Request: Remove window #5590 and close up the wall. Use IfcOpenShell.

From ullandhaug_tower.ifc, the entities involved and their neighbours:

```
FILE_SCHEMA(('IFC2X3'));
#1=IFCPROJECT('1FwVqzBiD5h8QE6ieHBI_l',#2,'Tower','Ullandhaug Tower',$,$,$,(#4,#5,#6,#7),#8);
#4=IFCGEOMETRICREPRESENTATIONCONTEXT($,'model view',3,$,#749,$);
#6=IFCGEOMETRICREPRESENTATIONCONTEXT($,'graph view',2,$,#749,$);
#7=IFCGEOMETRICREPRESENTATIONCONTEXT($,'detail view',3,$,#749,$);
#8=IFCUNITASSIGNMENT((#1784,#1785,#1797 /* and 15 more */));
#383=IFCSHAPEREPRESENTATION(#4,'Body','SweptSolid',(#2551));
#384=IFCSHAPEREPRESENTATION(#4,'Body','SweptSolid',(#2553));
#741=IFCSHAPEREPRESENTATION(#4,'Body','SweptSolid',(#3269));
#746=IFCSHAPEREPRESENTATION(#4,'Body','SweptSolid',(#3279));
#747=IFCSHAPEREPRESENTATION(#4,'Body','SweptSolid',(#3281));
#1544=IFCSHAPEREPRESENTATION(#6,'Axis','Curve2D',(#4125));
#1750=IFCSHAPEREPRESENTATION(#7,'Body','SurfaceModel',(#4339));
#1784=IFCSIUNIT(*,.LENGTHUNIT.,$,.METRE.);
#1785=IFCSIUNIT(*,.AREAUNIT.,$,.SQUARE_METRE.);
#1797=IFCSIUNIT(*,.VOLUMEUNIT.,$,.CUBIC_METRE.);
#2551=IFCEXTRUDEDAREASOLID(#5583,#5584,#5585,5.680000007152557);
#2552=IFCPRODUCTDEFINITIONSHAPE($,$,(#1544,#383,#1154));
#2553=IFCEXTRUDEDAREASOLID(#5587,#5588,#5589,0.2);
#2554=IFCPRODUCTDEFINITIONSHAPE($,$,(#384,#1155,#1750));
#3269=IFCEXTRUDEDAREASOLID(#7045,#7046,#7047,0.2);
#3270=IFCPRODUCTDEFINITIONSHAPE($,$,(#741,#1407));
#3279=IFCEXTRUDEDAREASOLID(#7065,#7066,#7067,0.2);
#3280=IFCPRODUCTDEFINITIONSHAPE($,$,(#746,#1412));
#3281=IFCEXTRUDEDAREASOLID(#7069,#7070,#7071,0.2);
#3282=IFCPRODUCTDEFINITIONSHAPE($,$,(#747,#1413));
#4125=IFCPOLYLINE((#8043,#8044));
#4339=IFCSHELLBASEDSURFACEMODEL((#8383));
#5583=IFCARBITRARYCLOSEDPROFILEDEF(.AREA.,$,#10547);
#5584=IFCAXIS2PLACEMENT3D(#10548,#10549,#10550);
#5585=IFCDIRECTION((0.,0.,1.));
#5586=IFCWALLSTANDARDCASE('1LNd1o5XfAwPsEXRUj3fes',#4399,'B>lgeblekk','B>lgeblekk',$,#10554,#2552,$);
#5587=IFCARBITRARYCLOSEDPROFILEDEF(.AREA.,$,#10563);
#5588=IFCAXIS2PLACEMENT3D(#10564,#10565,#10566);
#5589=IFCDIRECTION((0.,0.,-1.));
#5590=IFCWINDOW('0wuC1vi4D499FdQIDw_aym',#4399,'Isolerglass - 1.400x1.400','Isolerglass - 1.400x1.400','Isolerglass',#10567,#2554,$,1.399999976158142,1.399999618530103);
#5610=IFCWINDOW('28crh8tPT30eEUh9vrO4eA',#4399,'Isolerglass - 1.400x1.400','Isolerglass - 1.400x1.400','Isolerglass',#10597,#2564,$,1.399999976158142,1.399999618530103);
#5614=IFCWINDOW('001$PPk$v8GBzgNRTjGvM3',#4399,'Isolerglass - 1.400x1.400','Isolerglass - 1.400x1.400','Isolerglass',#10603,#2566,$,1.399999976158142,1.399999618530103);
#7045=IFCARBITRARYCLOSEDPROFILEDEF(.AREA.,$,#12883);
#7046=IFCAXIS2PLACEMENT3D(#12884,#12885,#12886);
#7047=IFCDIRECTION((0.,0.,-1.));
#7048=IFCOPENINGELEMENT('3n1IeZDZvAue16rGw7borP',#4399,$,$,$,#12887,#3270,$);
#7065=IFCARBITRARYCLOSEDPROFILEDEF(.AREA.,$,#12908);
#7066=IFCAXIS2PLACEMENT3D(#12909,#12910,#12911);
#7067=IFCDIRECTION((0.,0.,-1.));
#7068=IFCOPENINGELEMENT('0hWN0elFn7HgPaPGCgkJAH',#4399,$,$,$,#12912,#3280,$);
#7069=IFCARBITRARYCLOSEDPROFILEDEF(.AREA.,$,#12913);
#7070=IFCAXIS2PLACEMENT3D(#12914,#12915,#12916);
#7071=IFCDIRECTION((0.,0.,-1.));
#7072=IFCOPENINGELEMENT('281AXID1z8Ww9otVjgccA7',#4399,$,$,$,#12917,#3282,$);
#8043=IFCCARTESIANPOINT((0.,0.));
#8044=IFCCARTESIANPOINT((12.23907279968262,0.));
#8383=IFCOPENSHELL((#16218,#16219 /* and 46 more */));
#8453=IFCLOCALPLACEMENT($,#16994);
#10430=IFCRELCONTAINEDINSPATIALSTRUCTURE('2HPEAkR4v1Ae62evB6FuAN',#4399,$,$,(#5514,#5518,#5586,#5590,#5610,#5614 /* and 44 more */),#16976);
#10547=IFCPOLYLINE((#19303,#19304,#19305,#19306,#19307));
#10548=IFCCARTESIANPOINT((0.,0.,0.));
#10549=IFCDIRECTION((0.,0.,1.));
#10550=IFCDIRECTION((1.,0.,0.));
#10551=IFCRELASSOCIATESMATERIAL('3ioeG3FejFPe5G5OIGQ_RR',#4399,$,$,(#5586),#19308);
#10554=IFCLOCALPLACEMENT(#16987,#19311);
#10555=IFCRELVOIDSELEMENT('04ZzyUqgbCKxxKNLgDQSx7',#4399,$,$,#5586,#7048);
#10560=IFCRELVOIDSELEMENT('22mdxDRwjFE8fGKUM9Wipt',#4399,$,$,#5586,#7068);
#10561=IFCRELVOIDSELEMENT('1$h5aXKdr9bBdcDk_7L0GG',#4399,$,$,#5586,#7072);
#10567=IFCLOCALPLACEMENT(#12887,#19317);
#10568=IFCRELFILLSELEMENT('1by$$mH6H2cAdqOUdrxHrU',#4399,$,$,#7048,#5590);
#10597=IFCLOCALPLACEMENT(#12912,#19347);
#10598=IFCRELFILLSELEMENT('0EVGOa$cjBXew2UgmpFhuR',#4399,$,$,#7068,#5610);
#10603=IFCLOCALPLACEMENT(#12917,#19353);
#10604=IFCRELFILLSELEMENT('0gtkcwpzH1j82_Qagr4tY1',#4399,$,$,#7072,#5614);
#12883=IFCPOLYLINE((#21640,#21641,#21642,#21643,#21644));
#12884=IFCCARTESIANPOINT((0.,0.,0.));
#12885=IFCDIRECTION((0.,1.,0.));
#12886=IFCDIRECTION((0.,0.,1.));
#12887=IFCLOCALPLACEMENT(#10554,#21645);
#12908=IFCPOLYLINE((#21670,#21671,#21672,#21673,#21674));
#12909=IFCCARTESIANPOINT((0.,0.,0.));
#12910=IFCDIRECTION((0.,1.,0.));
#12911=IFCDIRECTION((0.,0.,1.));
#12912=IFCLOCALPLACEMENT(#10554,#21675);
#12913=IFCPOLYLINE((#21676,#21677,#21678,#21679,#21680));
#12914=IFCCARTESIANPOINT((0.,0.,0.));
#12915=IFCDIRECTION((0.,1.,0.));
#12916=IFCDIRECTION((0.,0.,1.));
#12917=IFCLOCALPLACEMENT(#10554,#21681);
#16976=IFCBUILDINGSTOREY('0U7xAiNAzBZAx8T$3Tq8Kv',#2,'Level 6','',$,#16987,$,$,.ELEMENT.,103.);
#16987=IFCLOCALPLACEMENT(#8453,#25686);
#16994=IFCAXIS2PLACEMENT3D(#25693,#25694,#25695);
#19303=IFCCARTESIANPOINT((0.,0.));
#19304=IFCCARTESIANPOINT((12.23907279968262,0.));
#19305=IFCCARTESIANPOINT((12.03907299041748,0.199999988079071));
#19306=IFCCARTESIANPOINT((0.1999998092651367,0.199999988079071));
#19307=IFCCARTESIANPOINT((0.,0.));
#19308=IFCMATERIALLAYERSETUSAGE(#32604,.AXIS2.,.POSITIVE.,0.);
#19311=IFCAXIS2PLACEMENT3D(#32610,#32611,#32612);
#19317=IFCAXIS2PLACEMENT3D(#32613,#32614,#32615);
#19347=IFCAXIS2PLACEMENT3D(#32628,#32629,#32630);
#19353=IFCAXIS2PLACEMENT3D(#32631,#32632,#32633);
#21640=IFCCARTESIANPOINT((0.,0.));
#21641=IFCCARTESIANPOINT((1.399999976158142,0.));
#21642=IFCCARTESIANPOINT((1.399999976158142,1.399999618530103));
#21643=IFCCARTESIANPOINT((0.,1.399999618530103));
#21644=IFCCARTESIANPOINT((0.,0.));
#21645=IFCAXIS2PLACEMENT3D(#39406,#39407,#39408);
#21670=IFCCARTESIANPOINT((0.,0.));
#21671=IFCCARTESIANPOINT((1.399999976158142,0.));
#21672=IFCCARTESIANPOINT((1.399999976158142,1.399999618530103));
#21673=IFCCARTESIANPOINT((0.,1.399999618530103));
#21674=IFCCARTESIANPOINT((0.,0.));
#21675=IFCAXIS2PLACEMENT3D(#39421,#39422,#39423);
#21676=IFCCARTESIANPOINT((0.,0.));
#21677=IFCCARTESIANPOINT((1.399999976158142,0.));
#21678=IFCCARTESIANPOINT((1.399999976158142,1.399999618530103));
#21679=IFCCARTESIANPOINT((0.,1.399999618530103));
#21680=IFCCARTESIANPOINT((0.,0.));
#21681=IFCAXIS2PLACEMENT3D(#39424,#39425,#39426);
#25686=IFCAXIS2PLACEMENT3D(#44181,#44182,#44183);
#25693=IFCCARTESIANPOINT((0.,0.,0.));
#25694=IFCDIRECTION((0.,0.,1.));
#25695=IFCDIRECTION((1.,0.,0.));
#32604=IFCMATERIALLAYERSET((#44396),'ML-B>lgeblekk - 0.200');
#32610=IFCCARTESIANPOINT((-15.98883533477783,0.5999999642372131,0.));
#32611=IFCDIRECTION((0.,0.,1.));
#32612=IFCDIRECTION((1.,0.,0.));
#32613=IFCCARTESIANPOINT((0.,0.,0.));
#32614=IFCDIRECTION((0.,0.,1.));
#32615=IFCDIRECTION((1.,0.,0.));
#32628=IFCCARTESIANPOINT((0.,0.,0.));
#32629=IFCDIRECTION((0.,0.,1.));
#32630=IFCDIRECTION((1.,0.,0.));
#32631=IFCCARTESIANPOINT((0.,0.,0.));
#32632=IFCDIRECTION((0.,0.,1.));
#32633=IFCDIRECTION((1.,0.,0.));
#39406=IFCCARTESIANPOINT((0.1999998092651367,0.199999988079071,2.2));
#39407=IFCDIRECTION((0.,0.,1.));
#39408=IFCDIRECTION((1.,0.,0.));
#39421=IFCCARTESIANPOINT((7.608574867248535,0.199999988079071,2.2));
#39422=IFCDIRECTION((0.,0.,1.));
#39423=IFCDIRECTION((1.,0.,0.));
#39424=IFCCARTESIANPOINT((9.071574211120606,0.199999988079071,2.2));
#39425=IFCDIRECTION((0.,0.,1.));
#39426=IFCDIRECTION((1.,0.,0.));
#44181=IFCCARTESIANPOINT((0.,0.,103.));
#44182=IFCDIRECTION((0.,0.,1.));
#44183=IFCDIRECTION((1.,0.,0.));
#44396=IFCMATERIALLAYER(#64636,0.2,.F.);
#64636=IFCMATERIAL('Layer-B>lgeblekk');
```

```python
import ifcopenshell
import ifcopenshell.api.feature
import ifcopenshell.api.root
import ifcopenshell.geom
import ifcopenshell.util.shape

model = ifcopenshell.open("ullandhaug_tower.ifc")
settings = ifcopenshell.geom.settings()


def volume(element):
    """Net volume in cubic metres, openings subtracted."""
    shape = ifcopenshell.geom.create_shape(settings, element)
    return ifcopenshell.util.shape.get_volume(shape.geometry)


window = model.by_guid("0wuC1vi4D499FdQIDw_aym")
opening = window.FillsVoids[0].RelatingOpeningElement
wall = opening.VoidsElements[0].RelatingBuildingElement
before = volume(wall)

ifcopenshell.api.root.remove_product(model, product=window)
ifcopenshell.api.feature.remove_feature(model, feature=opening)

after = volume(wall)

print(f"wall volume {before:.3f} -> {after:.3f} m3")

model.write("ullandhaug_tower_updated.ifc")
```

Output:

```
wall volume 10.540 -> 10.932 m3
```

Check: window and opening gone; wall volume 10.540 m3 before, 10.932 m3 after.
